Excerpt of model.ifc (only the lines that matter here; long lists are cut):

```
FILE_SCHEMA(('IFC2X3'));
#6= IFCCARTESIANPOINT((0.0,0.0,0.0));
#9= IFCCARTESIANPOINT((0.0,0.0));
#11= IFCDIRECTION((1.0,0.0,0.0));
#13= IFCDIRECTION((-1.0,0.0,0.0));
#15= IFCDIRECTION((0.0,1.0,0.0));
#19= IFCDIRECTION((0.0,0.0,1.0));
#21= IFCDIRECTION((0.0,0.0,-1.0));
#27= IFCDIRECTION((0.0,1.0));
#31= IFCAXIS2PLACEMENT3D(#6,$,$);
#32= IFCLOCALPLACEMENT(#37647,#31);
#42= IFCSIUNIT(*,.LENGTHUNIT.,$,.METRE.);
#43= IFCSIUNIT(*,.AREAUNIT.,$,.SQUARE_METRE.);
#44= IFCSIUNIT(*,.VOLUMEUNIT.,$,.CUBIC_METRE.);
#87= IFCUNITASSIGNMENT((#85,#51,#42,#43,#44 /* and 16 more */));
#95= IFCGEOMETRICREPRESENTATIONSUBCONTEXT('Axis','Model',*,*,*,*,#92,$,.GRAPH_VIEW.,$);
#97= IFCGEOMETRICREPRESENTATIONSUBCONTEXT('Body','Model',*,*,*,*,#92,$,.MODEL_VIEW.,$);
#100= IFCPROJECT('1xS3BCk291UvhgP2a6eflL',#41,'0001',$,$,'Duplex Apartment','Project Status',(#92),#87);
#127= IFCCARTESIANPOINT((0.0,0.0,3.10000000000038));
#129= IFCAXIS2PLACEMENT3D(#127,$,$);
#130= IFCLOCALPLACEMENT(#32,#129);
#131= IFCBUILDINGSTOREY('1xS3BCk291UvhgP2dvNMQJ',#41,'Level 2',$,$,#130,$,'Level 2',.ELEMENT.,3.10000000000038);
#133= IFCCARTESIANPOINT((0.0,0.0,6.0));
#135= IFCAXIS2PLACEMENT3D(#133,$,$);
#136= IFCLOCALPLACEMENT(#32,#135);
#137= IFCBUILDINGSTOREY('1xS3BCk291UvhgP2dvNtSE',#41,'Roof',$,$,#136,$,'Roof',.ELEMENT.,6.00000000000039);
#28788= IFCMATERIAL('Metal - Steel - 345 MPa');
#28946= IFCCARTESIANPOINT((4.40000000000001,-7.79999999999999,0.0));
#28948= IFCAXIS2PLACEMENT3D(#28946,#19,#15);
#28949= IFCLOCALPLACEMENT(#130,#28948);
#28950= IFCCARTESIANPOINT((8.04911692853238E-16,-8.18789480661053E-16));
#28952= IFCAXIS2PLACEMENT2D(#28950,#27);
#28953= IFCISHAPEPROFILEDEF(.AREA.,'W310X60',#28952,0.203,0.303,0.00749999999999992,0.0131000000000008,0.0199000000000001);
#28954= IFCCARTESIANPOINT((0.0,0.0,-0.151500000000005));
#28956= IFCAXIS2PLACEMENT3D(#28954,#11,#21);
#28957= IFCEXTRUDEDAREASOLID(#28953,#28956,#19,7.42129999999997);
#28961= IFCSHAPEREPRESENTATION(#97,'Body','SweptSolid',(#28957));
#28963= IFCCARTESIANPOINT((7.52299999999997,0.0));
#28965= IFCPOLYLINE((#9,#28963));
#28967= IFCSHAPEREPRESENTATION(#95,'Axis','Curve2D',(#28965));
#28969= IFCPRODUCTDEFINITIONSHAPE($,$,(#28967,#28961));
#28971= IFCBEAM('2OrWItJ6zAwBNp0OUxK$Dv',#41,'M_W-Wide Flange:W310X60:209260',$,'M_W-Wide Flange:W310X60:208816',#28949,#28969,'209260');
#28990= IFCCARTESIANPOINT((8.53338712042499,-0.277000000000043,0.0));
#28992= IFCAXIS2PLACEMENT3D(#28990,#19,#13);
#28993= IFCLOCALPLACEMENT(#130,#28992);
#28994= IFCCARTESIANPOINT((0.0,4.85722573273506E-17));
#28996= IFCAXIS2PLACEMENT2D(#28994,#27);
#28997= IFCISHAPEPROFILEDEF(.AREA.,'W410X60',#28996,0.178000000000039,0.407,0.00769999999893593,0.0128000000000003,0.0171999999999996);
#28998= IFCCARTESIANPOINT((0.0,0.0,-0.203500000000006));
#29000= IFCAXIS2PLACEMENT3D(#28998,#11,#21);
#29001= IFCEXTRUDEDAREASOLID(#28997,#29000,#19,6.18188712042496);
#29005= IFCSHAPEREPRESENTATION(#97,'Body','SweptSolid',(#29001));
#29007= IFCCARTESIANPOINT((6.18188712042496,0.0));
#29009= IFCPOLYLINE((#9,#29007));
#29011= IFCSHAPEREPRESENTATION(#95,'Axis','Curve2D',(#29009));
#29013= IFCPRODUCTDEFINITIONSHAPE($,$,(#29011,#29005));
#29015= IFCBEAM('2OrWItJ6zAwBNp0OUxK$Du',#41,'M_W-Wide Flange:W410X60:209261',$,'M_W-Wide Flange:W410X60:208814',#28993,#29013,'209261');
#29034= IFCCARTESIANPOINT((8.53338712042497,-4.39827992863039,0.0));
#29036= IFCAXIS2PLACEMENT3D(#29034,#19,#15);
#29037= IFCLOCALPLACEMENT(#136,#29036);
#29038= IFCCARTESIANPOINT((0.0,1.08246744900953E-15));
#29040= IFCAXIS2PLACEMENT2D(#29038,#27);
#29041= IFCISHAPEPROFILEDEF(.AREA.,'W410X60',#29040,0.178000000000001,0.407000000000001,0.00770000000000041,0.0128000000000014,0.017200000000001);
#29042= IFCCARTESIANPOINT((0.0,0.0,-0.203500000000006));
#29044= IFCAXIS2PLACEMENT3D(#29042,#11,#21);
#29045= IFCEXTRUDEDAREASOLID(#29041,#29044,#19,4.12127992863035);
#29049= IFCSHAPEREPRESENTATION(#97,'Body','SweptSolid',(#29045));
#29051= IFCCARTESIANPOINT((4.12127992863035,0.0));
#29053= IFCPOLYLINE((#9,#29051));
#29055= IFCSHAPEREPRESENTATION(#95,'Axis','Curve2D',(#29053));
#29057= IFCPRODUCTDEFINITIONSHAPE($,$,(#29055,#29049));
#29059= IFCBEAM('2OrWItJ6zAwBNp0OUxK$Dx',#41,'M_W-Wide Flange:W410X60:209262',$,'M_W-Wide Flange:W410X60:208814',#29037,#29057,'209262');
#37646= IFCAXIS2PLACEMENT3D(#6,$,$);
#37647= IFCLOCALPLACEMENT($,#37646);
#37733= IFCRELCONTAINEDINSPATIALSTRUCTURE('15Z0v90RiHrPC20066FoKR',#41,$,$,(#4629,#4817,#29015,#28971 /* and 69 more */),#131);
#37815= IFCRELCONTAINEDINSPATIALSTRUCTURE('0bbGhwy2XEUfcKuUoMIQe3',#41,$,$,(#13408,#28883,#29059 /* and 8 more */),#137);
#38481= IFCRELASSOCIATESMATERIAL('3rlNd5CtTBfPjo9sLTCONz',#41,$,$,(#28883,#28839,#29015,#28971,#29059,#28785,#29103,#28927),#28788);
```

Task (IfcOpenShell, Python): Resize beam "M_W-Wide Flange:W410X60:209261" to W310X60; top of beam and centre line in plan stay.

```python
import ifcopenshell
import ifcopenshell.util.element
import ifcopenshell.util.representation

model = ifcopenshell.open("model.ifc")

member = model.by_guid("2OrWItJ6zAwBNp0OUxK$Du")
source = next(p for p in model.by_type("IfcIShapeProfileDef") if p.ProfileName == "W310X60")

body = ifcopenshell.util.representation.get_representation(member, "Model", "Body")
solid = body.Items[0]
old_profile = solid.SweptArea

# Copy the section's sizes but keep this member's own profile position.
profile = ifcopenshell.util.element.copy(model, source)
# Profiles are centred, so shift by half the change in depth to hold the top.
shift = (old_profile.OverallDepth - profile.OverallDepth) / 2
x, y = old_profile.Position.Location.Coordinates
up = (-1.0, 0.0)  # upwards, in the solid's own plane
location = model.createIfcCartesianPoint((x + up[0] * shift, y + up[1] * shift))
profile.Position = model.createIfcAxis2Placement2D(location, old_profile.Position.RefDirection)
solid.SweptArea = profile
if not model.get_total_inverses(old_profile):
    ifcopenshell.util.element.remove_deep2(model, old_profile)
member.Name = member.Name.replace("W410X60", "W310X60")
member.ObjectType = member.ObjectType.replace("W410X60", "W310X60")

print(solid.SweptArea)

model.write("model_updated.ifc")
```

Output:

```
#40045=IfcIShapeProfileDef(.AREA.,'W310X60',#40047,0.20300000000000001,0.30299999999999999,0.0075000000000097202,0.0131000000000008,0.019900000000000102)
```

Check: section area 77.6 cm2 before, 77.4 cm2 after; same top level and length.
